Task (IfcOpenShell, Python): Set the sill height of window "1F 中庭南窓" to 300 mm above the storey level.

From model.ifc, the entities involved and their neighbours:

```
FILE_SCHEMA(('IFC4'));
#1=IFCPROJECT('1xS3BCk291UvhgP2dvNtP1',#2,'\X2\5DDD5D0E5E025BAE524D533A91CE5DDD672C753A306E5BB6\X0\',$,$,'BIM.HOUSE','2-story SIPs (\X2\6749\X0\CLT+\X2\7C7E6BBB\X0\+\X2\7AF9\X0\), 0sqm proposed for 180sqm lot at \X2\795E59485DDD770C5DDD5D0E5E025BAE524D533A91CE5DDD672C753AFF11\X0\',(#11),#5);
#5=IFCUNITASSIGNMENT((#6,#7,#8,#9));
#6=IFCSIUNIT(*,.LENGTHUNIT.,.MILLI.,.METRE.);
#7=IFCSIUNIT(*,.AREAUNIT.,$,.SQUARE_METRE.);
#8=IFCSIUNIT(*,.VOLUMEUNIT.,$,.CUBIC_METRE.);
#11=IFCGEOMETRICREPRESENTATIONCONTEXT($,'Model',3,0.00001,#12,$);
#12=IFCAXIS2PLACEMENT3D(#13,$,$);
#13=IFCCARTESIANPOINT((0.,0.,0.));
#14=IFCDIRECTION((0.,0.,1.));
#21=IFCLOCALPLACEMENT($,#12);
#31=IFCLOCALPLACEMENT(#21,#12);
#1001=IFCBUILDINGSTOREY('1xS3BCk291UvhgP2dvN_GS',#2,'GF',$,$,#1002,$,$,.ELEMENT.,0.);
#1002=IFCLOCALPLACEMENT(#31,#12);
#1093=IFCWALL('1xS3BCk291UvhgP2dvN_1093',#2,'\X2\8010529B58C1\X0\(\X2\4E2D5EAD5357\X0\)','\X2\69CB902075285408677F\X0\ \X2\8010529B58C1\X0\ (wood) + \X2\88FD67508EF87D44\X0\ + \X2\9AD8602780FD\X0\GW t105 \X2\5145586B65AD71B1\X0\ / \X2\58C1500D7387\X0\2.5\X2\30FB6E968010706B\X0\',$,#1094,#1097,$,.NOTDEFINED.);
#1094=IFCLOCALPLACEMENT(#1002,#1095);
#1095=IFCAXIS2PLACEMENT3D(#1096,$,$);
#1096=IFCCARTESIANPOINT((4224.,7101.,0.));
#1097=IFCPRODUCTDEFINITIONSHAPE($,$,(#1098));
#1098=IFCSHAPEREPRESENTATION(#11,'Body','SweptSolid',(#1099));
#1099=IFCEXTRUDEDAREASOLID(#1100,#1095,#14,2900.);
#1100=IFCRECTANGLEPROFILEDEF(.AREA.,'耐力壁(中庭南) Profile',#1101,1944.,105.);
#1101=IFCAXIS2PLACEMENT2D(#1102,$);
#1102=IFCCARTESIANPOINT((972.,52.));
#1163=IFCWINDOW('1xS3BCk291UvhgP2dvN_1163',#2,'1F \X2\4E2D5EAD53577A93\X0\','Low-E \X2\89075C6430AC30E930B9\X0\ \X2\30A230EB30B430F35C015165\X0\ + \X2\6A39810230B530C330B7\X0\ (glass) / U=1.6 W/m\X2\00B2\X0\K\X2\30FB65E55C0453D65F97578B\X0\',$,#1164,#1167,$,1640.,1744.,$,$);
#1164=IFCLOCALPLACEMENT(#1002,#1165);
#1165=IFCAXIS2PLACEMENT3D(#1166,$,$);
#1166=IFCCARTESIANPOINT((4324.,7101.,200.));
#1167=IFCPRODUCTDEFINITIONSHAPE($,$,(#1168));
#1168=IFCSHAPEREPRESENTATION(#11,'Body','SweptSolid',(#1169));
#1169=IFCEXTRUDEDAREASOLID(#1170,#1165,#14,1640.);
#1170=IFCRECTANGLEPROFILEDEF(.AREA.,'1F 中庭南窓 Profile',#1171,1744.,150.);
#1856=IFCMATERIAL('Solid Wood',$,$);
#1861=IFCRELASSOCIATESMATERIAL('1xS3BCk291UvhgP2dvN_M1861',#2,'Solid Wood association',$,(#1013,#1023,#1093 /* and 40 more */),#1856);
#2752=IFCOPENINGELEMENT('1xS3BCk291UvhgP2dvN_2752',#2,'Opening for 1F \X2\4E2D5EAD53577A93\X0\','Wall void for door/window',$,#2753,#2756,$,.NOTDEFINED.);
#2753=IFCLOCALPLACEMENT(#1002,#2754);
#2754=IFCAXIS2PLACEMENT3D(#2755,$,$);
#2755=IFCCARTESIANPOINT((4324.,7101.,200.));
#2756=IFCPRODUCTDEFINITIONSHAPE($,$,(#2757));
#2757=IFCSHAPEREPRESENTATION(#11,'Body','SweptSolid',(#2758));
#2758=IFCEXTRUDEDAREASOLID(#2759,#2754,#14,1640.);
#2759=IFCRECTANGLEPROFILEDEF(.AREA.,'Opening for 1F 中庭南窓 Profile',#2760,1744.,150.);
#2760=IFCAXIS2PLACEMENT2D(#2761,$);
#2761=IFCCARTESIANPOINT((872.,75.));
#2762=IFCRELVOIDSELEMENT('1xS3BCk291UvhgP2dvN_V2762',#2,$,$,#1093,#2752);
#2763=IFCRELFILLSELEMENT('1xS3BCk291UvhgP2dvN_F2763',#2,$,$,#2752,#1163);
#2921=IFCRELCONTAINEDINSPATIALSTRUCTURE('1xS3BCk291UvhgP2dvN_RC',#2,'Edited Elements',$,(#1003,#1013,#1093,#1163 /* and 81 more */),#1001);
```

```python
import numpy as np
import ifcopenshell
import ifcopenshell.api.geometry
import ifcopenshell.geom
import ifcopenshell.util.element
import ifcopenshell.util.placement
import ifcopenshell.util.shape
import ifcopenshell.util.unit

model = ifcopenshell.open("model.ifc")
unit_scale = ifcopenshell.util.unit.calculate_unit_scale(model)

window = model.by_id(1163)
opening = window.FillsVoids[0].RelatingOpeningElement
storey = ifcopenshell.util.element.get_container(window, ifc_class="IfcBuildingStorey")
level = ifcopenshell.util.placement.get_local_placement(storey.ObjectPlacement)[2, 3]

# The opening's origin need not be at the sill, so measure its lowest point.
shape = ifcopenshell.geom.create_shape(ifcopenshell.geom.settings(), opening)
bottom = ifcopenshell.util.shape.get_shape_bottom_elevation(shape, shape.geometry) / unit_scale
dz = level + 0.3 / unit_scale - bottom

shift = np.array([0.0, 0.0, dz])
# The window is not placed relative to its opening, so move both.
for product in (opening, window):
    matrix = ifcopenshell.util.placement.get_local_placement(product.ObjectPlacement)
    matrix[:3, 3] += shift
    ifcopenshell.api.geometry.edit_object_placement(model, product=product, matrix=matrix, is_si=False)

print(f"moved by {dz * unit_scale:+.3f} m")

model.write("model-out.ifc")
```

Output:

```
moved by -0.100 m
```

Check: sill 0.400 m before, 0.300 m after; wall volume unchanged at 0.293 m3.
